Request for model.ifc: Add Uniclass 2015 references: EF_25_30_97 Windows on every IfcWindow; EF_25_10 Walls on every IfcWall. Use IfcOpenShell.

First a look at what the model holds.

```python
import ifcopenshell

model = ifcopenshell.open("model.ifc")
print(model.schema)
print("classifications:", [c.Name for c in model.by_type("IfcClassification")])
for ifc_class in ("IfcDoor", "IfcRoof", "IfcStair", "IfcWall", "IfcWindow"):
    print(ifc_class, len(model.by_type(ifc_class)))
```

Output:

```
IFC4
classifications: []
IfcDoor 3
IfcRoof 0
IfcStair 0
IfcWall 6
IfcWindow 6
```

```python
import ifcopenshell
import ifcopenshell.api.classification

model = ifcopenshell.open("model.ifc")

system = ifcopenshell.api.classification.add_classification(model, classification="Uniclass 2015")

codes = {
    "IfcWindow": ("EF_25_30_97", "Windows"),
    "IfcWall": ("EF_25_10", "Walls"),
}
for ifc_class, (code, name) in codes.items():
    products = model.by_type(ifc_class)
    ifcopenshell.api.classification.add_reference(
        model, products=products, classification=system, identification=code, name=name
    )
    print(code, len(products))

model.write("model_updated.ifc")
```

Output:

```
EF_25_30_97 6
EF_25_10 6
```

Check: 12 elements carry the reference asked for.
